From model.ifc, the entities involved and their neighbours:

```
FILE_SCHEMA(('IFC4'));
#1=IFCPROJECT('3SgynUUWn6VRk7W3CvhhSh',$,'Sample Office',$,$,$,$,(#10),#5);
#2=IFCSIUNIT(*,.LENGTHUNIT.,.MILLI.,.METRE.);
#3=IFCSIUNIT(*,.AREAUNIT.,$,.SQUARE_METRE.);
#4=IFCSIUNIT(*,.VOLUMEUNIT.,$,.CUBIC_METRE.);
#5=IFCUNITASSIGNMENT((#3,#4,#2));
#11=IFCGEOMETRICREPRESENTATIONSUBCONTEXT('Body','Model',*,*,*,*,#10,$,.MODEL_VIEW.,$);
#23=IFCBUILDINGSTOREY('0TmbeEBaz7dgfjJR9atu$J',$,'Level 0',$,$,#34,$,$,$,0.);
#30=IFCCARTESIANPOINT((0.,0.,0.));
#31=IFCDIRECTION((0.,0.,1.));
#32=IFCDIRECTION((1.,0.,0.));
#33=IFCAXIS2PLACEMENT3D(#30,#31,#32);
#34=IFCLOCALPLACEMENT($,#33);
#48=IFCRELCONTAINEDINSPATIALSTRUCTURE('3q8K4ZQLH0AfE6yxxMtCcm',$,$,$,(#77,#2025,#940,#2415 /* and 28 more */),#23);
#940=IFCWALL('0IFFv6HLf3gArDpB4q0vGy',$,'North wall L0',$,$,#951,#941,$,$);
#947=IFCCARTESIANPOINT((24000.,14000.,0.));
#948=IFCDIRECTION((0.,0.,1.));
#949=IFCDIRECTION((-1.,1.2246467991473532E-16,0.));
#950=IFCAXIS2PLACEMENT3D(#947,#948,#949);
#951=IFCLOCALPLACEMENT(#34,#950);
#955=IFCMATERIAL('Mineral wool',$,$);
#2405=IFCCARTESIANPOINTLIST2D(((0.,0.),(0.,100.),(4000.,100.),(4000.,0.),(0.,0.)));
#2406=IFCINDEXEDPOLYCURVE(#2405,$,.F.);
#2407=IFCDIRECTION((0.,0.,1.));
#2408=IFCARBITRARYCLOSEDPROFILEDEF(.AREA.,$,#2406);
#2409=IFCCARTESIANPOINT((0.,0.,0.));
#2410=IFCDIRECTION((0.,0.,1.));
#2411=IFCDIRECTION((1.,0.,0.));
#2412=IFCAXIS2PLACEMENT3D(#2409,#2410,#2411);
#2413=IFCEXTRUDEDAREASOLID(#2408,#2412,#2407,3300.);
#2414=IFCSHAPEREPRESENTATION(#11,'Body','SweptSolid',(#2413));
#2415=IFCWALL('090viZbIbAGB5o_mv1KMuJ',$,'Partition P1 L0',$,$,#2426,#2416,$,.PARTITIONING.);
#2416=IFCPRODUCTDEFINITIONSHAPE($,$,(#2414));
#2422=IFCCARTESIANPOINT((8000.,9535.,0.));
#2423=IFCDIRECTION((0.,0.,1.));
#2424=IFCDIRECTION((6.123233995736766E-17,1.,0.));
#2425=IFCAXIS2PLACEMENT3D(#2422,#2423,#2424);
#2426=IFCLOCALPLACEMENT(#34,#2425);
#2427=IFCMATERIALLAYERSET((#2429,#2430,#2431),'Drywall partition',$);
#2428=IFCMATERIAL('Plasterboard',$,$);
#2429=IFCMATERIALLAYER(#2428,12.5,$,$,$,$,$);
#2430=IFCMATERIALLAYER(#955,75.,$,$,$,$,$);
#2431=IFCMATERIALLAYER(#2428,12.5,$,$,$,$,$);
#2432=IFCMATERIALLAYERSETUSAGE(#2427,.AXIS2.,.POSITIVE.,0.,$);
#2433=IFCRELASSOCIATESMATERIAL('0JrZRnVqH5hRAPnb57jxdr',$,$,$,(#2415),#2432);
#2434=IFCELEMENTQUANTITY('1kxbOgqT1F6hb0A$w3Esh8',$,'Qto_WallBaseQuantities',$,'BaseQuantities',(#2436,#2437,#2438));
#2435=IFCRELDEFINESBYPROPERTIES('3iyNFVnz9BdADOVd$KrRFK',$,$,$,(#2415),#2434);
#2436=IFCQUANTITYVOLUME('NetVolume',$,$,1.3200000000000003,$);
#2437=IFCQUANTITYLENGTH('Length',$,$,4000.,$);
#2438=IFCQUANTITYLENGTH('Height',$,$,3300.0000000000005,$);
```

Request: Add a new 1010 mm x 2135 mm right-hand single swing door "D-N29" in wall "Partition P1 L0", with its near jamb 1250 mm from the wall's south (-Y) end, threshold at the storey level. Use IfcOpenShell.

```python
import numpy as np
import ifcopenshell
import ifcopenshell.api.feature
import ifcopenshell.api.geometry
import ifcopenshell.api.pset
import ifcopenshell.api.root
import ifcopenshell.api.spatial
import ifcopenshell.geom
import ifcopenshell.util.element
import ifcopenshell.util.placement
import ifcopenshell.util.representation
import ifcopenshell.util.shape
import ifcopenshell.util.unit

model = ifcopenshell.open("model.ifc")
unit_scale = ifcopenshell.util.unit.calculate_unit_scale(model)
volume_scale = ifcopenshell.util.unit.calculate_unit_scale(model, "VOLUMEUNIT")
settings = ifcopenshell.geom.settings()


def volume(element):
    """Net volume in cubic metres, openings subtracted."""
    shape = ifcopenshell.geom.create_shape(settings, element)
    return ifcopenshell.util.shape.get_volume(shape.geometry)


wall = model.by_guid("090viZbIbAGB5o_mv1KMuJ")
storey = ifcopenshell.util.element.get_container(wall, ifc_class="IfcBuildingStorey")
context = ifcopenshell.util.representation.get_context(model, "Model", "Body", "MODEL_VIEW")
before = volume(wall)

width, height, from_end, sill = 1.01, 2.135, 1.25, 0.0  # metres

# The wall runs along its own X axis, and the end named is its -X end.
wall_shape = ifcopenshell.geom.create_shape(settings, wall)
x, y, z = ifcopenshell.util.shape.get_vertices(wall_shape.geometry).T
start = x.min() + from_end
face, thickness = float(y.min()), float(y.max() - y.min())
wall_matrix = ifcopenshell.util.placement.get_local_placement(wall.ObjectPlacement)
level = ifcopenshell.util.placement.get_local_placement(storey.ObjectPlacement)[2, 3]


def in_wall(x, y):
    """Placement at x, y metres in the wall's axes, at sill height."""
    matrix = wall_matrix.copy()
    matrix[:, 3] = wall_matrix @ np.array([x / unit_scale, y / unit_scale, 0.0, 1.0])
    matrix[2, 3] = level + sill / unit_scale
    return matrix


# Opening: a box that overshoots both wall faces by 50 mm.
opening = ifcopenshell.api.root.create_entity(model, ifc_class="IfcOpeningElement", predefined_type="OPENING")
box = ifcopenshell.api.geometry.add_wall_representation(
    model, context=context, length=width, height=height, thickness=thickness + 0.1
)
ifcopenshell.api.geometry.assign_representation(model, product=opening, representation=box)
ifcopenshell.api.geometry.edit_object_placement(model, product=opening, matrix=in_wall(start, face - 0.05), is_si=False)
ifcopenshell.api.feature.add_feature(model, feature=opening, element=wall)

door = ifcopenshell.api.root.create_entity(model, ifc_class="IfcDoor", name="D-N29", predefined_type="DOOR")
door.OverallWidth, door.OverallHeight = width / unit_scale, height / unit_scale
door.OperationType = "SINGLE_SWING_RIGHT"
body = ifcopenshell.api.geometry.add_door_representation(
    model,
    context=context,
    overall_width=door.OverallWidth,
    overall_height=door.OverallHeight,
    operation_type="SINGLE_SWING_RIGHT",
    lining_properties={"LiningDepth": thickness / unit_scale, "ThresholdDepth": thickness / unit_scale},
)
ifcopenshell.api.geometry.assign_representation(model, product=door, representation=body)
ifcopenshell.api.spatial.assign_container(model, products=[door], relating_structure=storey)
ifcopenshell.api.feature.add_filling(model, opening=opening, element=door)

# The lining spans the wall, so the door starts at the wall face.
ifcopenshell.api.geometry.edit_object_placement(model, product=door, matrix=in_wall(start, face), is_si=False)

after = volume(wall)

# Update the wall's stored quantities.
qto = model.by_id(ifcopenshell.util.element.get_pset(wall, "Qto_WallBaseQuantities", should_inherit=False)["id"])
ifcopenshell.api.pset.edit_qto(model, qto=qto, properties={"NetVolume": after / volume_scale})

print(f"wall volume {before:.3f} -> {after:.3f} m3")

model.write("model_edited.ifc")
```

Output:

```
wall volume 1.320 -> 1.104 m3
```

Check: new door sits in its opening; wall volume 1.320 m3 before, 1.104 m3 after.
